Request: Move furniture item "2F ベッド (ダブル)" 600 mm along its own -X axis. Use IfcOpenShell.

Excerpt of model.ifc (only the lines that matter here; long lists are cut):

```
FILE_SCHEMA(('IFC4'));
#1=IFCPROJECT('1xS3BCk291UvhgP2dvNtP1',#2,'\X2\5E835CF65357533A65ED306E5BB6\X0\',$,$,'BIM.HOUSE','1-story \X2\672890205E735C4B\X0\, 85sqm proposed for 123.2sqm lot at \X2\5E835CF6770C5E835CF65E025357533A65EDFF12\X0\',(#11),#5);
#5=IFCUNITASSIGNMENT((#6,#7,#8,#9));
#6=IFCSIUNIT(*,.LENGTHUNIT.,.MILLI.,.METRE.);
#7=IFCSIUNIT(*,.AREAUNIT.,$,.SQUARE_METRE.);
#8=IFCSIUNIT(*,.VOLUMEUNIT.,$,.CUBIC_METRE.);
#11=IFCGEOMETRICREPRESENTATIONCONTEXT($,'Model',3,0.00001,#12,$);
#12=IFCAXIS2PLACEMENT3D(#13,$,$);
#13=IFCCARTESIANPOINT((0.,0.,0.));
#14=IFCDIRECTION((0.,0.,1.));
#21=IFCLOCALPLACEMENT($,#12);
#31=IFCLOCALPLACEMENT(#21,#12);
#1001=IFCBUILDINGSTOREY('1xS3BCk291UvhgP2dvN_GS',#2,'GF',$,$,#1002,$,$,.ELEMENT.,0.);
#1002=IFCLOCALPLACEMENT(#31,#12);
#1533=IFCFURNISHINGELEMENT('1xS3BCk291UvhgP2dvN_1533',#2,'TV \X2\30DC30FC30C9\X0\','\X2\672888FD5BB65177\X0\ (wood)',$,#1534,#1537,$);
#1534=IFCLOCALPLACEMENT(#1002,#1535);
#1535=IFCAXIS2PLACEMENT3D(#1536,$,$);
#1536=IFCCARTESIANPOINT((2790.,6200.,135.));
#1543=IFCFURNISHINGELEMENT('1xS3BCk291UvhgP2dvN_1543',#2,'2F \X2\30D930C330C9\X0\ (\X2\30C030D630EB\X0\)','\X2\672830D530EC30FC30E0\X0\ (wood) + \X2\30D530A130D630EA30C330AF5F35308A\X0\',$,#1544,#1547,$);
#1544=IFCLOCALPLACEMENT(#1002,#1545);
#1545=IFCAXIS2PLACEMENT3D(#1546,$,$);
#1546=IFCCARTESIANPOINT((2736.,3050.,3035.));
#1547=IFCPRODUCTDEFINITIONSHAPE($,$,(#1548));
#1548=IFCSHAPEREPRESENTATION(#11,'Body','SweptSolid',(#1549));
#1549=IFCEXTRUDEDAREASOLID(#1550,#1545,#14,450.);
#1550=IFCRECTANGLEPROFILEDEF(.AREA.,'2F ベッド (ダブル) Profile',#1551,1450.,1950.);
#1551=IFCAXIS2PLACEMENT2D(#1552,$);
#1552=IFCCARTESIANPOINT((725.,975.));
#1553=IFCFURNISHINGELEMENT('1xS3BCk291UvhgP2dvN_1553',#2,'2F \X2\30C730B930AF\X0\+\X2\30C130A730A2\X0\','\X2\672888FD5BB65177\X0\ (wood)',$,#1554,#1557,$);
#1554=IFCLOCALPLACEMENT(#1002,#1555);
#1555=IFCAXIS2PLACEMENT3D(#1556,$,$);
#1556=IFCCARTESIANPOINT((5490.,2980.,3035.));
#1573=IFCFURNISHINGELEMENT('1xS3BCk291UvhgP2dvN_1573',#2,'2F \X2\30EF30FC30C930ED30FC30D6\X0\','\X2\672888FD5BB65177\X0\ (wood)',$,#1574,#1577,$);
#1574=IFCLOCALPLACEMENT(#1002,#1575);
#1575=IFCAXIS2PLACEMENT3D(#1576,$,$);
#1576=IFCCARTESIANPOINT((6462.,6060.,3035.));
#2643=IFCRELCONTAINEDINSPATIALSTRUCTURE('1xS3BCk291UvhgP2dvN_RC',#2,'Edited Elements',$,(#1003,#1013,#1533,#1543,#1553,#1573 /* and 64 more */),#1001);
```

```python
import ifcopenshell
import ifcopenshell.api.geometry
import ifcopenshell.util.placement

model = ifcopenshell.open("model.ifc")

item = model.by_guid("1xS3BCk291UvhgP2dvN_1543")
matrix = ifcopenshell.util.placement.get_local_placement(item.ObjectPlacement)
matrix[:3, 3] -= matrix[:3, 0] * 600.0
ifcopenshell.api.geometry.edit_object_placement(model, product=item, matrix=matrix, is_si=False)

print(ifcopenshell.util.placement.get_local_placement(item.ObjectPlacement).round(3) + 0.0)

model.write("model_rev.ifc")
```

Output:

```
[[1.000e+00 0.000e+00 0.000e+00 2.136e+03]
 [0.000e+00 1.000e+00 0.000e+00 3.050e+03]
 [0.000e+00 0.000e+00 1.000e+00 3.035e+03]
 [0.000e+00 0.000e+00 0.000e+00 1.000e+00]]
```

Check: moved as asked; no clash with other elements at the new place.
